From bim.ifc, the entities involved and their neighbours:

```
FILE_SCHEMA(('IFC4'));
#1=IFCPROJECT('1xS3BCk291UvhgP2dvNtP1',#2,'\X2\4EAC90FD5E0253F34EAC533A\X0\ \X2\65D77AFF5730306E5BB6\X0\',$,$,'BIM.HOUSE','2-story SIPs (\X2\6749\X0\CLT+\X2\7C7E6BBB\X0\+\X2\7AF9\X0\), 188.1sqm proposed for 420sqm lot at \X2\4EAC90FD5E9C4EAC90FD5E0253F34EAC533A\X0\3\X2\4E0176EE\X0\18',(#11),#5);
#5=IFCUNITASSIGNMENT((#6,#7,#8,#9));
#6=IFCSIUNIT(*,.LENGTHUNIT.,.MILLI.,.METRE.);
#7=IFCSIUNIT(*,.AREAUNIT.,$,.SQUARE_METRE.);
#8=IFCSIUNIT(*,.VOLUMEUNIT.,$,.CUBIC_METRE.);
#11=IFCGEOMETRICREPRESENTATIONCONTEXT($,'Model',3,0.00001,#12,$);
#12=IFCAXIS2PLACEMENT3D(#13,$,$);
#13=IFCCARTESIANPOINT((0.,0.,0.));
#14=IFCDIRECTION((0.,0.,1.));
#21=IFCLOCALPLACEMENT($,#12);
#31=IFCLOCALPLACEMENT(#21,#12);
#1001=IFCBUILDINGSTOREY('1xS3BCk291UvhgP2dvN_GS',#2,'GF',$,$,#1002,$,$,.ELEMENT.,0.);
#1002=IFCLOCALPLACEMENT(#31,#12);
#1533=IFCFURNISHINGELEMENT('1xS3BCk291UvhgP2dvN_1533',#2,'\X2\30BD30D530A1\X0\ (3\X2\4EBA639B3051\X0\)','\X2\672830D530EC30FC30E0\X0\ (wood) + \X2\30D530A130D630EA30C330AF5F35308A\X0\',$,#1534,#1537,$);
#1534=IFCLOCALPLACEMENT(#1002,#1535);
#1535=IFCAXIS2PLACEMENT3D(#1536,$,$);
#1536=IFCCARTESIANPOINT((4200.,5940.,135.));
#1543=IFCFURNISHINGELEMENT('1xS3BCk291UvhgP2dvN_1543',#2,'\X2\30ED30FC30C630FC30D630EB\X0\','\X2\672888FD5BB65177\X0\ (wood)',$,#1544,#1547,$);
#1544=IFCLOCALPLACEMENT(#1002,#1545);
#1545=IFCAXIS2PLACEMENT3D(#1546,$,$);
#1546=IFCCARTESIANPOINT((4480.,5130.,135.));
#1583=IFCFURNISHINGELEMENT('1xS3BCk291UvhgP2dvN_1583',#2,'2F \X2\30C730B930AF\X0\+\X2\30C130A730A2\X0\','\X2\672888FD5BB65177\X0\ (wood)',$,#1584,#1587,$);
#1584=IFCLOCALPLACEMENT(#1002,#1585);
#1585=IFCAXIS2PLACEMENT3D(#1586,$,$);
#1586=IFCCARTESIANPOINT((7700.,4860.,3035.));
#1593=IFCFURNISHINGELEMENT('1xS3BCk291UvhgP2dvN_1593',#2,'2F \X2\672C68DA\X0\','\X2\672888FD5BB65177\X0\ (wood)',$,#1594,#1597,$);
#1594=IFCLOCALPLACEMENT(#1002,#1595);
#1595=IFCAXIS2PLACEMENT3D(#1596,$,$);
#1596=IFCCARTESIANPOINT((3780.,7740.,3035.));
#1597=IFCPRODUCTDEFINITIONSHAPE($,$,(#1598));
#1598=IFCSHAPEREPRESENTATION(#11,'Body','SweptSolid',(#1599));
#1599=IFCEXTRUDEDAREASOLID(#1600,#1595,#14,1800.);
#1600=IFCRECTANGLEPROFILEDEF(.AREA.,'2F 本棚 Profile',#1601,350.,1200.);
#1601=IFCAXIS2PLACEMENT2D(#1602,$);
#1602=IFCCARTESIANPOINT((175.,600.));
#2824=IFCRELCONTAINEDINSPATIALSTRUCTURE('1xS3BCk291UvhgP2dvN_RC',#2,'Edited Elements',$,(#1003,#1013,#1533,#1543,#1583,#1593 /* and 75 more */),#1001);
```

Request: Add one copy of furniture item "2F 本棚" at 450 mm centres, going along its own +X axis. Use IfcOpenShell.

```python
import ifcopenshell
import ifcopenshell.api.geometry
import ifcopenshell.api.root
import ifcopenshell.util.element
import ifcopenshell.util.placement
import ifcopenshell.util.unit

model = ifcopenshell.open("bim.ifc")
unit_scale = ifcopenshell.util.unit.calculate_unit_scale(model)


def reuse_history(source, copy):
    """copy_class also copies each property set's owner history, people and application; keep the originals."""
    for rel in copy.IsDefinedBy:
        if rel.is_a("IfcRelDefinesByProperties") and (history := rel.RelatingPropertyDefinition.OwnerHistory):
            rel.RelatingPropertyDefinition.OwnerHistory = source.OwnerHistory
            ifcopenshell.util.element.remove_deep2(model, history)


source = model.by_guid("1xS3BCk291UvhgP2dvN_1593")
base = ifcopenshell.util.placement.get_local_placement(source.ObjectPlacement)
step = base[:3, 0] * 0.45 / unit_scale

for i in range(1, 2):
    copy = ifcopenshell.api.root.copy_class(model, product=source)
    copy.Representation = ifcopenshell.util.element.copy_deep(
        model, source.Representation, exclude=["IfcGeometricRepresentationContext", "IfcRepresentationMap"]
    )
    reuse_history(source, copy)
    matrix = base.copy()
    matrix[:3, 3] += i * step
    print("added at", matrix[:3, 3].round(3) + 0.0)
    ifcopenshell.api.geometry.edit_object_placement(model, product=copy, matrix=matrix, is_si=False)

model.write("bim_updated.ifc")
```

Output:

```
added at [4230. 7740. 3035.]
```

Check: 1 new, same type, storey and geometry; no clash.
